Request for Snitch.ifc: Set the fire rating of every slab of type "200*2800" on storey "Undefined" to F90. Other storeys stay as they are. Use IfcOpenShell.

First a look at what the model holds.

```python
import ifcopenshell
import ifcopenshell.util.element

model = ifcopenshell.open("Snitch.ifc")
print(model.schema)
storey = next(s for s in model.by_type("IfcBuildingStorey") if s.Name == "Undefined")
slabs = [e for e in ifcopenshell.util.element.get_decomposition(storey) if e.is_a("IfcSlab")]
seen = {}
for e in slabs:
    element_type = ifcopenshell.util.element.get_type(e)
    key = (element_type.Name if element_type != e and element_type else None, ifcopenshell.util.element.get_pset(e, "Pset_SlabCommon", "FireRating"))
    seen[key] = seen.get(key, 0) + 1
for (name, value), count in sorted(seen.items(), key=str):
    print(count, "x", name, "|", value)
```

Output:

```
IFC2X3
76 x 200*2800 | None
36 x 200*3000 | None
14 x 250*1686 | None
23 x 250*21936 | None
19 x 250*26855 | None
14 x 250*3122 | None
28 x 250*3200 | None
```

```python
import ifcopenshell
import ifcopenshell.api.pset
import ifcopenshell.util.element

model = ifcopenshell.open("Snitch.ifc")

storey = next(s for s in model.by_type("IfcBuildingStorey") if s.Name == "Undefined")
slabs = [e for e in ifcopenshell.util.element.get_decomposition(storey) if e.is_a("IfcSlab")]

count = 0
for e in slabs:
    element_type = ifcopenshell.util.element.get_type(e)
    if element_type in (None, e) or element_type.Name != "200*2800":
        continue
    found = ifcopenshell.util.element.get_pset(e, "Pset_SlabCommon", should_inherit=False)
    if found:
        pset = model.by_id(found["id"])
        if len(ifcopenshell.util.element.get_elements_by_pset(pset)) > 1:
            pset = ifcopenshell.api.pset.unshare_pset(model, products=[e], pset=pset)[0]
    else:
        pset = ifcopenshell.api.pset.add_pset(model, product=e, name="Pset_SlabCommon")
    ifcopenshell.api.pset.edit_pset(model, pset=pset, properties={"FireRating": "F90"})
    count += 1

print(count, "slabs updated")

model.write("Snitch_v2.ifc")
```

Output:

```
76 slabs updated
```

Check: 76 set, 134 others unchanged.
